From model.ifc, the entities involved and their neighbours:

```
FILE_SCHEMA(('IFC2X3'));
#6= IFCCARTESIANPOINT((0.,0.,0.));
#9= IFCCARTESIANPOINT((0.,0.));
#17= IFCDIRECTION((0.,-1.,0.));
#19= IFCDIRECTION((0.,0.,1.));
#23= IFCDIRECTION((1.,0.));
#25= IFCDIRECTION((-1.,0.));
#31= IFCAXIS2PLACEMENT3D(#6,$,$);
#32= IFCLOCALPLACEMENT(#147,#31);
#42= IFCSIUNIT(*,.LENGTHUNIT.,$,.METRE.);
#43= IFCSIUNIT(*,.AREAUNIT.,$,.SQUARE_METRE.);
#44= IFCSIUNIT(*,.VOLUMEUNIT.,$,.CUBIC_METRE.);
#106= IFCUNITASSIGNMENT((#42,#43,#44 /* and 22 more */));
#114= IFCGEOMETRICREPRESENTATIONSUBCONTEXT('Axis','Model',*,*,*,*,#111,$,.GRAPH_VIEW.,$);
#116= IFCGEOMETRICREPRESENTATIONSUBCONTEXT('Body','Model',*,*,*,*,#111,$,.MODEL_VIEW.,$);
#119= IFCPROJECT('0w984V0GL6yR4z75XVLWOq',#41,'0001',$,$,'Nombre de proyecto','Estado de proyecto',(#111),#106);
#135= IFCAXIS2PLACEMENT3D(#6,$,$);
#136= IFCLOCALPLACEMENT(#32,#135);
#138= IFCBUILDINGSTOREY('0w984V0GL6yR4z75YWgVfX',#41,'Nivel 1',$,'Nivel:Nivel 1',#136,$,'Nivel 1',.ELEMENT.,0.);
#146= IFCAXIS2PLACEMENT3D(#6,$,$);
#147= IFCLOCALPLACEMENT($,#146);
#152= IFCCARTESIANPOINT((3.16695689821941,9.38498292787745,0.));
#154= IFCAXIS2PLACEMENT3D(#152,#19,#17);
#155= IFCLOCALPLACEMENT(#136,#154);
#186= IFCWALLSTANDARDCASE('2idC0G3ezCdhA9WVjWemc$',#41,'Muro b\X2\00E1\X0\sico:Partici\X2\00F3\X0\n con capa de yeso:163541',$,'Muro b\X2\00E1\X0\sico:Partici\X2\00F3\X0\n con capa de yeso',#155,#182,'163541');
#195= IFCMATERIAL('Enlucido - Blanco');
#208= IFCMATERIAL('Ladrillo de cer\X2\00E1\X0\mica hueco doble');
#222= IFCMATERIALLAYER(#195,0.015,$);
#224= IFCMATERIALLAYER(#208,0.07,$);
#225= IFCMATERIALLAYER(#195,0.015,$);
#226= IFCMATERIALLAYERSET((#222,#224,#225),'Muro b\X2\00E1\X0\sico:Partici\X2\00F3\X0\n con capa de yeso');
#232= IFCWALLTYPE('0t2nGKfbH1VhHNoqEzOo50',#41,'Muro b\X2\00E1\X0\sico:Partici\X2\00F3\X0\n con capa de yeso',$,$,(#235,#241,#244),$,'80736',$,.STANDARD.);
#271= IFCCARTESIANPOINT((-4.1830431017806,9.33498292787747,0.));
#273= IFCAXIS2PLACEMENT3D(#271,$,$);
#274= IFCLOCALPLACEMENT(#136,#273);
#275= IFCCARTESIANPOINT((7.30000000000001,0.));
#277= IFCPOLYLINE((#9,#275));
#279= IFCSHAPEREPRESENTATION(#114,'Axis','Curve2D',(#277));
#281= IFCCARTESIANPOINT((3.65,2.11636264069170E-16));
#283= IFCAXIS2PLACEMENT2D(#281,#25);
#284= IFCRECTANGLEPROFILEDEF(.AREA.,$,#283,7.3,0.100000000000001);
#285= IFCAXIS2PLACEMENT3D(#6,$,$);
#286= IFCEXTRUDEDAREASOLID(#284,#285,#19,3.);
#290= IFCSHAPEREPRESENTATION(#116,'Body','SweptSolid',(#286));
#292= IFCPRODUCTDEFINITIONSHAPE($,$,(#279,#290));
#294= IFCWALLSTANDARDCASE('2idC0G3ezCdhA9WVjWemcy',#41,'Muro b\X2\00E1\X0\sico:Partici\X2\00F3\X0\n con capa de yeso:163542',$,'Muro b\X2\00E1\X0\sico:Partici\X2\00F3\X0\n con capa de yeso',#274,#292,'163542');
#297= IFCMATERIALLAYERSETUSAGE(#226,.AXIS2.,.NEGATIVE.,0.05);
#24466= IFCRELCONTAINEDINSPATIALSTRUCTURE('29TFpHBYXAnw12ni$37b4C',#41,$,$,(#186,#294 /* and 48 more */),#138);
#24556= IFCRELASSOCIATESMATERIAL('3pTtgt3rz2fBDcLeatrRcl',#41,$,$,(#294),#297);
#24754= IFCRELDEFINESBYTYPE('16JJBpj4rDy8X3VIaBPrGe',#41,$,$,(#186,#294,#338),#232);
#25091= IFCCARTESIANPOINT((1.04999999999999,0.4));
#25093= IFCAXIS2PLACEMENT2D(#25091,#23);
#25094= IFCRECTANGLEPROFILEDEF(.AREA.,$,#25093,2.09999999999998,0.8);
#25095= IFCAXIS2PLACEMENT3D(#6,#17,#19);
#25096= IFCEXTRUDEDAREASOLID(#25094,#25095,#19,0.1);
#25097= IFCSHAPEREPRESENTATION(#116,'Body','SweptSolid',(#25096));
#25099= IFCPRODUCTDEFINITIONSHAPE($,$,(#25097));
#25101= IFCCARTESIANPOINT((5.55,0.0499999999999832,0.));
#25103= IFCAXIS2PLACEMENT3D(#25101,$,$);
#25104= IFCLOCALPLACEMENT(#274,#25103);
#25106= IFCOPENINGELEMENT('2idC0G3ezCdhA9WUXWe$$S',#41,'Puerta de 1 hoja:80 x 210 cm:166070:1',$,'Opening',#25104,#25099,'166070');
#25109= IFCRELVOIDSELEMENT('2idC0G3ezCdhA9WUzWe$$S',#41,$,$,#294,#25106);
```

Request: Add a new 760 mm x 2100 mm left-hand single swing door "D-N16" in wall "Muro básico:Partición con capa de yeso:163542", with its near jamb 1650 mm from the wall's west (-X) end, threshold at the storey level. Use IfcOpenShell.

```python
import numpy as np
import ifcopenshell
import ifcopenshell.api.feature
import ifcopenshell.api.geometry
import ifcopenshell.api.root
import ifcopenshell.api.spatial
import ifcopenshell.api.type
import ifcopenshell.geom
import ifcopenshell.util.element
import ifcopenshell.util.placement
import ifcopenshell.util.representation
import ifcopenshell.util.shape
import ifcopenshell.util.unit

model = ifcopenshell.open("model.ifc")
unit_scale = ifcopenshell.util.unit.calculate_unit_scale(model)
settings = ifcopenshell.geom.settings()


def volume(element):
    """Net volume in cubic metres, openings subtracted."""
    shape = ifcopenshell.geom.create_shape(settings, element)
    return ifcopenshell.util.shape.get_volume(shape.geometry)


wall = model.by_guid("2idC0G3ezCdhA9WVjWemcy")
storey = ifcopenshell.util.element.get_container(wall, ifc_class="IfcBuildingStorey")
context = ifcopenshell.util.representation.get_context(model, "Model", "Body", "MODEL_VIEW")
before = volume(wall)

width, height, from_end, sill = 0.76, 2.1, 1.65, 0.0  # metres

# The wall runs along its own X axis, and the end named is its -X end.
wall_shape = ifcopenshell.geom.create_shape(settings, wall)
x, y, z = ifcopenshell.util.shape.get_vertices(wall_shape.geometry).T
start = x.min() + from_end
face, thickness = float(y.min()), float(y.max() - y.min())
wall_matrix = ifcopenshell.util.placement.get_local_placement(wall.ObjectPlacement)
level = ifcopenshell.util.placement.get_local_placement(storey.ObjectPlacement)[2, 3]


def in_wall(x, y):
    """Placement at x, y metres in the wall's axes, at sill height."""
    matrix = wall_matrix.copy()
    matrix[:, 3] = wall_matrix @ np.array([x / unit_scale, y / unit_scale, 0.0, 1.0])
    matrix[2, 3] = level + sill / unit_scale
    return matrix


# Opening: a box that overshoots both wall faces by 50 mm.
opening = ifcopenshell.api.root.create_entity(model, ifc_class="IfcOpeningElement")
box = ifcopenshell.api.geometry.add_wall_representation(
    model, context=context, length=width, height=height, thickness=thickness + 0.1
)
ifcopenshell.api.geometry.assign_representation(model, product=opening, representation=box)
ifcopenshell.api.geometry.edit_object_placement(model, product=opening, matrix=in_wall(start, face - 0.05), is_si=False)
ifcopenshell.api.feature.add_feature(model, feature=opening, element=wall)

door = ifcopenshell.api.root.create_entity(model, ifc_class="IfcDoor", name="D-N16")
door.OverallWidth, door.OverallHeight = width / unit_scale, height / unit_scale
body = ifcopenshell.api.geometry.add_door_representation(
    model,
    context=context,
    overall_width=door.OverallWidth,
    overall_height=door.OverallHeight,
    operation_type="SINGLE_SWING_LEFT",
    lining_properties={"LiningDepth": thickness / unit_scale, "ThresholdDepth": thickness / unit_scale},
)
ifcopenshell.api.geometry.assign_representation(model, product=door, representation=body)
ifcopenshell.api.spatial.assign_container(model, products=[door], relating_structure=storey)
fills = ifcopenshell.api.feature.add_filling(model, opening=opening, element=door)
fills.OwnerHistory = door.OwnerHistory  # required in IFC2X3

# IFC2X3 keeps the operation on the door style.
style = ifcopenshell.api.root.create_entity(model, ifc_class="IfcDoorStyle", name="D-N16")
style.OperationType, style.ConstructionType = "SINGLE_SWING_LEFT", "NOTDEFINED"
style.ParameterTakesPrecedence = style.Sizeable = False
ifcopenshell.api.type.assign_type(model, related_objects=[door], relating_type=style)

# The lining spans the wall, so the door starts at the wall face.
ifcopenshell.api.geometry.edit_object_placement(model, product=door, matrix=in_wall(start, face), is_si=False)

after = volume(wall)

print(f"wall volume {before:.3f} -> {after:.3f} m3")

model.write("model-out.ifc")
```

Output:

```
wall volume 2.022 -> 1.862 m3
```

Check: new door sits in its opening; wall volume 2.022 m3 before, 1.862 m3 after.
